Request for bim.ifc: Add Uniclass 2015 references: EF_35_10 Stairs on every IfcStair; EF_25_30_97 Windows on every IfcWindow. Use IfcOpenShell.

First a look at what the model holds.

```python
import ifcopenshell

model = ifcopenshell.open("bim.ifc")
print(model.schema)
print("classifications:", [c.Name for c in model.by_type("IfcClassification")])
for ifc_class in ("IfcDoor", "IfcRoof", "IfcStair", "IfcWall", "IfcWindow"):
    print(ifc_class, len(model.by_type(ifc_class)))
```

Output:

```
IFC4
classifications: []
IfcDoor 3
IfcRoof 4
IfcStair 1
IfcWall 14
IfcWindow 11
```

```python
import ifcopenshell
import ifcopenshell.api.classification

model = ifcopenshell.open("bim.ifc")

system = ifcopenshell.api.classification.add_classification(model, classification="Uniclass 2015")

codes = {
    "IfcStair": ("EF_35_10", "Stairs"),
    "IfcWindow": ("EF_25_30_97", "Windows"),
}
for ifc_class, (code, name) in codes.items():
    products = model.by_type(ifc_class)
    ifcopenshell.api.classification.add_reference(
        model, products=products, classification=system, identification=code, name=name
    )
    print(code, len(products))

model.write("bim_edited.ifc")
```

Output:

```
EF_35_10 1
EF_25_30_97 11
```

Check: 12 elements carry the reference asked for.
